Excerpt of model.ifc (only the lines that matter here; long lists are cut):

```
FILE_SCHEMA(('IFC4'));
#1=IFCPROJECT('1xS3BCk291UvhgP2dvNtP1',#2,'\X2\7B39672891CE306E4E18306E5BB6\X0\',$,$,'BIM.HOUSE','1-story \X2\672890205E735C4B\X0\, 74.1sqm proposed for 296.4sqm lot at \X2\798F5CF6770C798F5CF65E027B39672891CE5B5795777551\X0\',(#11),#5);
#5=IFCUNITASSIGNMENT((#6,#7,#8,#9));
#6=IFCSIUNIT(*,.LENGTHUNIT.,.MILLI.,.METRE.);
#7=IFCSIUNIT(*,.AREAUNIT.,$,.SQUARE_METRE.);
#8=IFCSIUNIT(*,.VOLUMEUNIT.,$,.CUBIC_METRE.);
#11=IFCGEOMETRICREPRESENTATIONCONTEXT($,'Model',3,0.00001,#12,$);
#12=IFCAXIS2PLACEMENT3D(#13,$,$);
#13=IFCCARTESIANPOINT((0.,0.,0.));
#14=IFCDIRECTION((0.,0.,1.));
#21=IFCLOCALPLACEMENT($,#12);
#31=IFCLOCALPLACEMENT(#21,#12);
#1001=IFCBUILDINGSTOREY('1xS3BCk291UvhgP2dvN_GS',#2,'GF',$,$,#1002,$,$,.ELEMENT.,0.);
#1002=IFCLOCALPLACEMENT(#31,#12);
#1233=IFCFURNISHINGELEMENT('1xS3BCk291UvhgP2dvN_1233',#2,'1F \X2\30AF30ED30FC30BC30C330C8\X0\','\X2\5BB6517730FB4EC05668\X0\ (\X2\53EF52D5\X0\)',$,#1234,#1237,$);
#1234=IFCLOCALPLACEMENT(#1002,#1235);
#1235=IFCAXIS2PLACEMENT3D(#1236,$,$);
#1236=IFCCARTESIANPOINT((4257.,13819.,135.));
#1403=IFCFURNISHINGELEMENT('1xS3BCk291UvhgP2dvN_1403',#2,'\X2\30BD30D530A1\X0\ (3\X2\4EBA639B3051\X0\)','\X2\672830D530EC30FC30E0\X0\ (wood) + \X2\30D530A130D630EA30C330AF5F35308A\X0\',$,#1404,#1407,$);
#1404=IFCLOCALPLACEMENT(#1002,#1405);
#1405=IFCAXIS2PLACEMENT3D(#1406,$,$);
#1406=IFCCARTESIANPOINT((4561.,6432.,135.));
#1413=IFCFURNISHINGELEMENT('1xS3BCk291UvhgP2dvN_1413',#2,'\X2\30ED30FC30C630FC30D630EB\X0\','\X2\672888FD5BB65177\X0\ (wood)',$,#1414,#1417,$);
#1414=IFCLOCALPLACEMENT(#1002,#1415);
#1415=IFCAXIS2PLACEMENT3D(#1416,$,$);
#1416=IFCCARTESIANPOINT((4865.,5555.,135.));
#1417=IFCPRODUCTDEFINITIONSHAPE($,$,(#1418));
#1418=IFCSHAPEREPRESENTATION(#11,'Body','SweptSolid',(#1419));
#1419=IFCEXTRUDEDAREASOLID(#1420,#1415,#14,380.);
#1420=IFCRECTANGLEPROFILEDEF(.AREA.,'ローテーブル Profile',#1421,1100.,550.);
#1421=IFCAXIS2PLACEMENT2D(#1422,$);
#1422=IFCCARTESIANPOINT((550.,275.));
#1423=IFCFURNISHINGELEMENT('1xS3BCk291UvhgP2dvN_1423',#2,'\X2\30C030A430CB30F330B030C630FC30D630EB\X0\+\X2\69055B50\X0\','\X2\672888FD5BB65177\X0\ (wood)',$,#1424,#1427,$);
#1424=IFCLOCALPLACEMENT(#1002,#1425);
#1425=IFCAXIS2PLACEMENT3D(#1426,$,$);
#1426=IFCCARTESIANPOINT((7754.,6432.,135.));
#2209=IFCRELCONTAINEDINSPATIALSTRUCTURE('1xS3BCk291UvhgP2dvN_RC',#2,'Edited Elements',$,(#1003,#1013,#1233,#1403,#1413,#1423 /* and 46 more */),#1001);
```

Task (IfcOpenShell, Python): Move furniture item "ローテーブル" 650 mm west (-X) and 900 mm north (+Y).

```python
import ifcopenshell
import ifcopenshell.api.geometry
import ifcopenshell.util.placement

model = ifcopenshell.open("model.ifc")

item = model.by_guid("1xS3BCk291UvhgP2dvN_1413")
matrix = ifcopenshell.util.placement.get_local_placement(item.ObjectPlacement)
matrix[0, 3] -= 650.0
matrix[1, 3] += 900.0
ifcopenshell.api.geometry.edit_object_placement(model, product=item, matrix=matrix, is_si=False)

print(ifcopenshell.util.placement.get_local_placement(item.ObjectPlacement).round(3) + 0.0)

model.write("model_edited.ifc")
```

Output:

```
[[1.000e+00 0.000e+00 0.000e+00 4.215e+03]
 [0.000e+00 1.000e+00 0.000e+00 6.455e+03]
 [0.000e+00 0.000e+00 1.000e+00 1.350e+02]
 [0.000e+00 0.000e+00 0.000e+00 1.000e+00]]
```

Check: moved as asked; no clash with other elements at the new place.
